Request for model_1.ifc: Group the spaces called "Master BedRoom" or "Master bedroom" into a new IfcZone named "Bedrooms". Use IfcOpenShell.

First a look at what the model holds.

```python
import ifcopenshell

model = ifcopenshell.open("model_1.ifc")
print(model.schema)
seen = {}
for space in model.by_type("IfcSpace"):
    seen[space.LongName] = seen.get(space.LongName, 0) + 1
for name, count in sorted(seen.items(), key=str):
    print(count, "x", name)
print("zones:", [z.Name for z in model.by_type("IfcZone")][:20])
```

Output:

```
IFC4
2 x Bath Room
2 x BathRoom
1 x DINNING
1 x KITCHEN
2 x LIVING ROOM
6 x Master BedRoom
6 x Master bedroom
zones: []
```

```python
import ifcopenshell
import ifcopenshell.api.group
import ifcopenshell.api.root

model = ifcopenshell.open("model_1.ifc")

names = {"Master BedRoom", "Master bedroom"}
spaces = [s for s in model.by_type("IfcSpace") if s.LongName in names]

zone = ifcopenshell.api.root.create_entity(model, ifc_class="IfcZone", name="Bedrooms")
ifcopenshell.api.group.assign_group(model, products=spaces, group=zone)
print(len(spaces), "spaces in", zone.Name)

model.write("model_1-out.ifc")
```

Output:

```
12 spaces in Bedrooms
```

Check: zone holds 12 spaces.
